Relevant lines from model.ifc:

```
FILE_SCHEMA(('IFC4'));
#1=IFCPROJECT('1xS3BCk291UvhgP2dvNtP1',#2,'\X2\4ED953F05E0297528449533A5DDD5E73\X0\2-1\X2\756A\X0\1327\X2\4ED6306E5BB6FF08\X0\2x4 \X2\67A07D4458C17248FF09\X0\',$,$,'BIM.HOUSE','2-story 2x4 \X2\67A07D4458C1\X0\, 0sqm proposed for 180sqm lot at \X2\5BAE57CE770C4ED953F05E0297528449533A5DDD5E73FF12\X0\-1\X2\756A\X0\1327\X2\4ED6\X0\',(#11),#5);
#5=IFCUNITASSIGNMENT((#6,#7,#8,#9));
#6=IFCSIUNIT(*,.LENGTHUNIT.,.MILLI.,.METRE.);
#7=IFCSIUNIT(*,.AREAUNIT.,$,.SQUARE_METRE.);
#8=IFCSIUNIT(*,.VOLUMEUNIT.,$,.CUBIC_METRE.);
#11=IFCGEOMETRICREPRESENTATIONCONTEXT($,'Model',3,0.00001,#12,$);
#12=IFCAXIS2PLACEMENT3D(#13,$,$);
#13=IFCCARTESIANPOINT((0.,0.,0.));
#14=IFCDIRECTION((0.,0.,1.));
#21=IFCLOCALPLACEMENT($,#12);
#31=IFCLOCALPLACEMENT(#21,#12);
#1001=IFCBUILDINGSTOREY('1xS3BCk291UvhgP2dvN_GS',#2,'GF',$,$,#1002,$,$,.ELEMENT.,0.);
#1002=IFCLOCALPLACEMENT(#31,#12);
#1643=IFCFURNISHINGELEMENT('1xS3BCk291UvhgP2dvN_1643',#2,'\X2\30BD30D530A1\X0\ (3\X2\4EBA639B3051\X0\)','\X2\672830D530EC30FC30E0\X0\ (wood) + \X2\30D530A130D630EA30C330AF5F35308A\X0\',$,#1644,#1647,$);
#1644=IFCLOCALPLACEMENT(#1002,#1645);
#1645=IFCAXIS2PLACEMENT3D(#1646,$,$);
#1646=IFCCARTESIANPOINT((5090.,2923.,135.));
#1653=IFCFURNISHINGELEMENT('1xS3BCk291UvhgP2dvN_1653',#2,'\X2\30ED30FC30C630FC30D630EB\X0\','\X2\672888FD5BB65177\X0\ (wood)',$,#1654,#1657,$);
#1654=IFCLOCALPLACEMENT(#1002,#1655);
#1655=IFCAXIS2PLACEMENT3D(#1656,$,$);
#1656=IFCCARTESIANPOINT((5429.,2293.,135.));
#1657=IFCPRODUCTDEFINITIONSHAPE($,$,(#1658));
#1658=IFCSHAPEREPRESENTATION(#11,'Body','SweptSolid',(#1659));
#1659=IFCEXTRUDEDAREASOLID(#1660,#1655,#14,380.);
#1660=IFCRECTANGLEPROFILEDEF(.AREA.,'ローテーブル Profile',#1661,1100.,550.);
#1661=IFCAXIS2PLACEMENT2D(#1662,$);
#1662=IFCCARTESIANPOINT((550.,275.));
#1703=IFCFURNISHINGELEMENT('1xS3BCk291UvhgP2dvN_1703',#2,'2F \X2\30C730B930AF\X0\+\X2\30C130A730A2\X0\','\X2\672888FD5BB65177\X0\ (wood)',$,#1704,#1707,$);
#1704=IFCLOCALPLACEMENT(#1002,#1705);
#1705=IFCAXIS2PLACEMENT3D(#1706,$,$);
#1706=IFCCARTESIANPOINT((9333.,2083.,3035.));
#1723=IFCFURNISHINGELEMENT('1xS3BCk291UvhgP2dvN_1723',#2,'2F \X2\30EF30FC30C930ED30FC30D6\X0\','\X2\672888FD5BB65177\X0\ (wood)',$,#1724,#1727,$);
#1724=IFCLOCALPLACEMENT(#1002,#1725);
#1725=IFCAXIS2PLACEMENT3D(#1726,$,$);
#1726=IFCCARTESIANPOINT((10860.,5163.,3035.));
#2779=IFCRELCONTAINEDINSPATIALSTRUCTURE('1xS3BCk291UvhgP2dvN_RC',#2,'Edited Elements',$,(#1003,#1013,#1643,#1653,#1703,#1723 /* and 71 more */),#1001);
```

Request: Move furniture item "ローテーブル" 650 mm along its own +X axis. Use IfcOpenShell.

```python
import ifcopenshell
import ifcopenshell.api.geometry
import ifcopenshell.util.placement
import ifcopenshell.util.unit

model = ifcopenshell.open("model.ifc")
unit_scale = ifcopenshell.util.unit.calculate_unit_scale(model)

item = model.by_guid("1xS3BCk291UvhgP2dvN_1653")
matrix = ifcopenshell.util.placement.get_local_placement(item.ObjectPlacement)
matrix[:3, 3] += matrix[:3, 0] * 0.65 / unit_scale
ifcopenshell.api.geometry.edit_object_placement(model, product=item, matrix=matrix, is_si=False)

print(ifcopenshell.util.placement.get_local_placement(item.ObjectPlacement).round(3) + 0.0)

model.write("model_updated.ifc")
```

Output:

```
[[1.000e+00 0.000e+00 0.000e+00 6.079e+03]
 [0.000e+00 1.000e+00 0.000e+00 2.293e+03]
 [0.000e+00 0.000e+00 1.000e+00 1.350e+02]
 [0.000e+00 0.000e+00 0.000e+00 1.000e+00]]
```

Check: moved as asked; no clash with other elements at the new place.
